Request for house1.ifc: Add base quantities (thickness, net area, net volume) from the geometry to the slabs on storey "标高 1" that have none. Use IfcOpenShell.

First a look at what the model holds.

```python
import ifcopenshell
import ifcopenshell.util.element
import ifcopenshell.util.unit

model = ifcopenshell.open("house1.ifc")
print(model.schema)
for unit_type in ("LENGTHUNIT", "AREAUNIT", "VOLUMEUNIT"):
    print(unit_type, ifcopenshell.util.unit.calculate_unit_scale(model, unit_type))
storey = next(s for s in model.by_type("IfcBuildingStorey") if s.Name == "标高 1")
slabs = [e for e in ifcopenshell.util.element.get_decomposition(storey) if e.is_a("IfcSlab")]
for e in sorted(slabs, key=lambda e: e.id()):
    print(e.id(), e.is_a(), e.Name, list(ifcopenshell.util.element.get_psets(e, qtos_only=True)), sep=" | ")
```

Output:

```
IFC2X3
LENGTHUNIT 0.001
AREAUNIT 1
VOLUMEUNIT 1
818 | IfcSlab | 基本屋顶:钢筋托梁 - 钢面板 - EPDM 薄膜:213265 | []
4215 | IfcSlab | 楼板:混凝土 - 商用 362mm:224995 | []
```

```python
import ifcopenshell
import ifcopenshell.api.pset
import ifcopenshell.geom
import ifcopenshell.util.element
import ifcopenshell.util.shape
import ifcopenshell.util.unit

model = ifcopenshell.open("house1.ifc")
unit_scale = ifcopenshell.util.unit.calculate_unit_scale(model)
area_scale = ifcopenshell.util.unit.calculate_unit_scale(model, "AREAUNIT")
volume_scale = ifcopenshell.util.unit.calculate_unit_scale(model, "VOLUMEUNIT")
settings = ifcopenshell.geom.settings()

storey = next(s for s in model.by_type("IfcBuildingStorey") if s.Name == "标高 1")
slabs = [e for e in ifcopenshell.util.element.get_decomposition(storey) if e.is_a("IfcSlab")]

for e in sorted(slabs, key=lambda e: e.id()):
    if ifcopenshell.util.element.get_psets(e, qtos_only=True, should_inherit=False):
        continue
    # Geometry comes back in metres, in the element's own axes.
    shape = ifcopenshell.geom.create_shape(settings, e)
    values = {
        "Width": ifcopenshell.util.shape.get_z(shape.geometry) / unit_scale,
        "NetArea": ifcopenshell.util.shape.get_footprint_area(shape.geometry) / area_scale,
        "NetVolume": ifcopenshell.util.shape.get_volume(shape.geometry) / volume_scale,
    }
    qto = ifcopenshell.api.pset.add_qto(model, product=e, name="BaseQuantities")
    ifcopenshell.api.pset.edit_qto(model, qto=qto, properties=values)
    print(e.id(), {k: round(v, 3) for k, v in values.items()})

model.write("house1_rev.ifc")
```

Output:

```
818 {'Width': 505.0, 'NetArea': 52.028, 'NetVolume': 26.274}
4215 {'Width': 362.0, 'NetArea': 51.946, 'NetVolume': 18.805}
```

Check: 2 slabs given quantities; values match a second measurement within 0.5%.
